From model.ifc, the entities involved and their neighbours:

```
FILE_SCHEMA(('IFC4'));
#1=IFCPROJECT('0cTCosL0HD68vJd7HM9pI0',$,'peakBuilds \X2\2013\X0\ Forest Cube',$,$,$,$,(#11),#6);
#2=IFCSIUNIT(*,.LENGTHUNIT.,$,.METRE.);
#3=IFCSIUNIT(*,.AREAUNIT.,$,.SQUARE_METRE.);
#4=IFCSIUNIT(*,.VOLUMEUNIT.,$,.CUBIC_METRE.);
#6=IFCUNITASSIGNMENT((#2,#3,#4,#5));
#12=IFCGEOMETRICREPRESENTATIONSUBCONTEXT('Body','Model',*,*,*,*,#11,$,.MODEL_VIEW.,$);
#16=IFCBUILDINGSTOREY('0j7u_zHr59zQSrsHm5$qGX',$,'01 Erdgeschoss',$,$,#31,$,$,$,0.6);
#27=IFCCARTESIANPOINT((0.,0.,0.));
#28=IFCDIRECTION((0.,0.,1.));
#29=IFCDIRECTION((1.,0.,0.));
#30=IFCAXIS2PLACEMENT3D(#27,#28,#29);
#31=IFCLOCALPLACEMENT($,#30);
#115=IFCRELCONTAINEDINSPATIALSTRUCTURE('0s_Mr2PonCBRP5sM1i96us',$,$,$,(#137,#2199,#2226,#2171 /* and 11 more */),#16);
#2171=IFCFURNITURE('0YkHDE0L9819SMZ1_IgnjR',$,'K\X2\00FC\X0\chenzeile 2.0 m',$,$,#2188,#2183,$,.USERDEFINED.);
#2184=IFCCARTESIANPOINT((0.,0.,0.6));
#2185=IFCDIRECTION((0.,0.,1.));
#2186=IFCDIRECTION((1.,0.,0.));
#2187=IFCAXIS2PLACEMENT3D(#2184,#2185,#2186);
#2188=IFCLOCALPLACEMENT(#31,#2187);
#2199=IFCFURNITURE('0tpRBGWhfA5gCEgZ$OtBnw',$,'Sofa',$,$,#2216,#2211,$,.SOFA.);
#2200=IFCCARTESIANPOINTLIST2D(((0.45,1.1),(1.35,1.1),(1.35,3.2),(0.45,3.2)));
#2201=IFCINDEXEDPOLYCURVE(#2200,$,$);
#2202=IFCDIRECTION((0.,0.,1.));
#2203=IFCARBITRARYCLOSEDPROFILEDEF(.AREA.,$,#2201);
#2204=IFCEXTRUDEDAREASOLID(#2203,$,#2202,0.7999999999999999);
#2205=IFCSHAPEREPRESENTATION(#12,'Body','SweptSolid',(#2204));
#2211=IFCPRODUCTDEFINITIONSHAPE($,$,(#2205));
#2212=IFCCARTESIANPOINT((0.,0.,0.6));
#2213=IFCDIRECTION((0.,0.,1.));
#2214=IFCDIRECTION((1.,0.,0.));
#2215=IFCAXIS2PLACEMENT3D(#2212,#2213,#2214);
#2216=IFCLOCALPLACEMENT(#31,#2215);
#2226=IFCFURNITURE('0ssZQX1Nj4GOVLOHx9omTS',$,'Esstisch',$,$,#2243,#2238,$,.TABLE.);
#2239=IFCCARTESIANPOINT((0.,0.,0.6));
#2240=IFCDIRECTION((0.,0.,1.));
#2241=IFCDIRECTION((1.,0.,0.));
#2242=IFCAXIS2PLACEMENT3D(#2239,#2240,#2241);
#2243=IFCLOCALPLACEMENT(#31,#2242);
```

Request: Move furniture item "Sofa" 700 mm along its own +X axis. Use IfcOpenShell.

```python
import ifcopenshell
import ifcopenshell.api.geometry
import ifcopenshell.util.placement

model = ifcopenshell.open("model.ifc")

item = model.by_guid("0tpRBGWhfA5gCEgZ$OtBnw")
matrix = ifcopenshell.util.placement.get_local_placement(item.ObjectPlacement)
matrix[:3, 3] += matrix[:3, 0] * 0.7
ifcopenshell.api.geometry.edit_object_placement(model, product=item, matrix=matrix, is_si=False)

print(ifcopenshell.util.placement.get_local_placement(item.ObjectPlacement).round(3) + 0.0)

model.write("model_v2.ifc")
```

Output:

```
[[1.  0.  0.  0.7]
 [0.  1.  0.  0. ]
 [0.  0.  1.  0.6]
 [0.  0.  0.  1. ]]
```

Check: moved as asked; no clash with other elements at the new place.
